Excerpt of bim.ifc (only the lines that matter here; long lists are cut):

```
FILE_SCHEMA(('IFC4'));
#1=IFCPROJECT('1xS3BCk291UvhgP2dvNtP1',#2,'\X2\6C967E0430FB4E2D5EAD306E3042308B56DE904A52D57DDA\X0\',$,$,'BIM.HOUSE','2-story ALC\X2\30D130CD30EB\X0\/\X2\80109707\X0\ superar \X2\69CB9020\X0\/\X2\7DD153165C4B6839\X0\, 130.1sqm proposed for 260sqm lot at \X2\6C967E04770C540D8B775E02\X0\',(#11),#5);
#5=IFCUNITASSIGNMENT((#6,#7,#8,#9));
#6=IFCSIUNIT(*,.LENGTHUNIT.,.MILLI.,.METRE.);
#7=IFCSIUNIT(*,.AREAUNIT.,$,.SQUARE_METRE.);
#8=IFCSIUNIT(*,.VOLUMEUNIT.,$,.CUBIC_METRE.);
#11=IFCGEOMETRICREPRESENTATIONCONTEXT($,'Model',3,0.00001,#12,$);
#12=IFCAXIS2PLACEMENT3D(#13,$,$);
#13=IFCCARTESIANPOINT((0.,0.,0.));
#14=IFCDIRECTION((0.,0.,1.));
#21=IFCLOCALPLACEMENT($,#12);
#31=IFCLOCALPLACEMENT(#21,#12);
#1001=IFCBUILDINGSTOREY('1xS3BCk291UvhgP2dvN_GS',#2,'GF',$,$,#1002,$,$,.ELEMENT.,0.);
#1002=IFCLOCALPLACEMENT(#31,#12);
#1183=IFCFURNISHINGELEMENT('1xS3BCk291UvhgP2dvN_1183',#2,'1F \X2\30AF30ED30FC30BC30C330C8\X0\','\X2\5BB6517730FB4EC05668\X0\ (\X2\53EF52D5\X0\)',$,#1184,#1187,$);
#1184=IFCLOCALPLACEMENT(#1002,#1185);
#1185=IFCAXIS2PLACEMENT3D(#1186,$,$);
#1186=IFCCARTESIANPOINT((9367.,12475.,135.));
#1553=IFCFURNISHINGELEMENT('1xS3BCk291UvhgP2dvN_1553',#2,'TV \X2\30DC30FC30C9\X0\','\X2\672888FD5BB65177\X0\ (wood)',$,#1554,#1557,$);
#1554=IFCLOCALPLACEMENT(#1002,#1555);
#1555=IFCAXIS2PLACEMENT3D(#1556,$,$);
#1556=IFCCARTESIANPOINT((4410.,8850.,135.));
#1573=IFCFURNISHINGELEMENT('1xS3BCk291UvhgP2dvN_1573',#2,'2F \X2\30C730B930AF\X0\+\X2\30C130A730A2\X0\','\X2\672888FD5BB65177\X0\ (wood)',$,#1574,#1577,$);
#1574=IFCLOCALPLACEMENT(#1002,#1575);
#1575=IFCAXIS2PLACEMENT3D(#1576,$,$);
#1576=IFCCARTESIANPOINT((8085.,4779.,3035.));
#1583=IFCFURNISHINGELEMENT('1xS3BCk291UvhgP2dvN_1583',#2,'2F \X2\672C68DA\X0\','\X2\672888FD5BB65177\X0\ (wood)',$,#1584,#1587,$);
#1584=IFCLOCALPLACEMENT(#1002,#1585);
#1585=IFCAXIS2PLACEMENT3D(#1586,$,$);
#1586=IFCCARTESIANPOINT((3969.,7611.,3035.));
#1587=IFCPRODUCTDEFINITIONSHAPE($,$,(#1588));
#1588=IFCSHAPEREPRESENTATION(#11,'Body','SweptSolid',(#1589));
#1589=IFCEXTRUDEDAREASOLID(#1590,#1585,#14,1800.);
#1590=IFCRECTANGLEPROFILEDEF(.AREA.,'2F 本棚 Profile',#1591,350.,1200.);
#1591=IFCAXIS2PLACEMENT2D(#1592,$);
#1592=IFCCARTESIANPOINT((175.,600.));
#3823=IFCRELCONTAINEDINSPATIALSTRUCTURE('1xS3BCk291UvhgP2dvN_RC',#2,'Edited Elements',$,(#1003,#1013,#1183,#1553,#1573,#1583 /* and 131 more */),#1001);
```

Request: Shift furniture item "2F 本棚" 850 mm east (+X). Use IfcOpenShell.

```python
import ifcopenshell
import ifcopenshell.api.geometry
import ifcopenshell.util.placement
import ifcopenshell.util.unit

model = ifcopenshell.open("bim.ifc")
unit_scale = ifcopenshell.util.unit.calculate_unit_scale(model)

item = model.by_id(1583)
matrix = ifcopenshell.util.placement.get_local_placement(item.ObjectPlacement)
matrix[0, 3] += 0.85 / unit_scale
ifcopenshell.api.geometry.edit_object_placement(model, product=item, matrix=matrix, is_si=False)

print(ifcopenshell.util.placement.get_local_placement(item.ObjectPlacement).round(3) + 0.0)

model.write("bim_updated.ifc")
```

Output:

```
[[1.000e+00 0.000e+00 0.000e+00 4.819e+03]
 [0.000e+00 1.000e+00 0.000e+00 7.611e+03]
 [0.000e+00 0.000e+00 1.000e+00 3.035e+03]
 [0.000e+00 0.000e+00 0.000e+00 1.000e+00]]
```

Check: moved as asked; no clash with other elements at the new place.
